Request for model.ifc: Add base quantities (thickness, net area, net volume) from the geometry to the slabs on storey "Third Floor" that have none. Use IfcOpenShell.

First a look at what the model holds.

```python
import ifcopenshell
import ifcopenshell.util.element
import ifcopenshell.util.unit

model = ifcopenshell.open("model.ifc")
print(model.schema)
for unit_type in ("LENGTHUNIT", "AREAUNIT", "VOLUMEUNIT"):
    print(unit_type, ifcopenshell.util.unit.calculate_unit_scale(model, unit_type))
storey = next(s for s in model.by_type("IfcBuildingStorey") if s.Name == "Third Floor")
slabs = [e for e in ifcopenshell.util.element.get_decomposition(storey) if e.is_a("IfcSlab")]
for e in sorted(slabs, key=lambda e: e.id()):
    print(e.id(), e.is_a(), e.Name, list(ifcopenshell.util.element.get_psets(e, qtos_only=True)), sep=" | ")
```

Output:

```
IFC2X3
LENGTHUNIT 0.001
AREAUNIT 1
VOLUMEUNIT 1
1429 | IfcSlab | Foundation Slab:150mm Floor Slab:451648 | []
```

```python
import ifcopenshell
import ifcopenshell.api.pset
import ifcopenshell.geom
import ifcopenshell.util.element
import ifcopenshell.util.shape
import ifcopenshell.util.unit

model = ifcopenshell.open("model.ifc")
unit_scale = ifcopenshell.util.unit.calculate_unit_scale(model)
area_scale = ifcopenshell.util.unit.calculate_unit_scale(model, "AREAUNIT")
volume_scale = ifcopenshell.util.unit.calculate_unit_scale(model, "VOLUMEUNIT")
settings = ifcopenshell.geom.settings()

storey = next(s for s in model.by_type("IfcBuildingStorey") if s.Name == "Third Floor")
slabs = [e for e in ifcopenshell.util.element.get_decomposition(storey) if e.is_a("IfcSlab")]

for e in sorted(slabs, key=lambda e: e.id()):
    if ifcopenshell.util.element.get_psets(e, qtos_only=True, should_inherit=False):
        continue
    # Geometry comes back in metres, in the element's own axes.
    shape = ifcopenshell.geom.create_shape(settings, e)
    values = {
        "Width": ifcopenshell.util.shape.get_z(shape.geometry) / unit_scale,
        "NetArea": ifcopenshell.util.shape.get_footprint_area(shape.geometry) / area_scale,
        "NetVolume": ifcopenshell.util.shape.get_volume(shape.geometry) / volume_scale,
    }
    qto = ifcopenshell.api.pset.add_qto(model, product=e, name="BaseQuantities")
    ifcopenshell.api.pset.edit_qto(model, qto=qto, properties=values)
    print(e.id(), {k: round(v, 3) for k, v in values.items()})

model.write("model_rev.ifc")
```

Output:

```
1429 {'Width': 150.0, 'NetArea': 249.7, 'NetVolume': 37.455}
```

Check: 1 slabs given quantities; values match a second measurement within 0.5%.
